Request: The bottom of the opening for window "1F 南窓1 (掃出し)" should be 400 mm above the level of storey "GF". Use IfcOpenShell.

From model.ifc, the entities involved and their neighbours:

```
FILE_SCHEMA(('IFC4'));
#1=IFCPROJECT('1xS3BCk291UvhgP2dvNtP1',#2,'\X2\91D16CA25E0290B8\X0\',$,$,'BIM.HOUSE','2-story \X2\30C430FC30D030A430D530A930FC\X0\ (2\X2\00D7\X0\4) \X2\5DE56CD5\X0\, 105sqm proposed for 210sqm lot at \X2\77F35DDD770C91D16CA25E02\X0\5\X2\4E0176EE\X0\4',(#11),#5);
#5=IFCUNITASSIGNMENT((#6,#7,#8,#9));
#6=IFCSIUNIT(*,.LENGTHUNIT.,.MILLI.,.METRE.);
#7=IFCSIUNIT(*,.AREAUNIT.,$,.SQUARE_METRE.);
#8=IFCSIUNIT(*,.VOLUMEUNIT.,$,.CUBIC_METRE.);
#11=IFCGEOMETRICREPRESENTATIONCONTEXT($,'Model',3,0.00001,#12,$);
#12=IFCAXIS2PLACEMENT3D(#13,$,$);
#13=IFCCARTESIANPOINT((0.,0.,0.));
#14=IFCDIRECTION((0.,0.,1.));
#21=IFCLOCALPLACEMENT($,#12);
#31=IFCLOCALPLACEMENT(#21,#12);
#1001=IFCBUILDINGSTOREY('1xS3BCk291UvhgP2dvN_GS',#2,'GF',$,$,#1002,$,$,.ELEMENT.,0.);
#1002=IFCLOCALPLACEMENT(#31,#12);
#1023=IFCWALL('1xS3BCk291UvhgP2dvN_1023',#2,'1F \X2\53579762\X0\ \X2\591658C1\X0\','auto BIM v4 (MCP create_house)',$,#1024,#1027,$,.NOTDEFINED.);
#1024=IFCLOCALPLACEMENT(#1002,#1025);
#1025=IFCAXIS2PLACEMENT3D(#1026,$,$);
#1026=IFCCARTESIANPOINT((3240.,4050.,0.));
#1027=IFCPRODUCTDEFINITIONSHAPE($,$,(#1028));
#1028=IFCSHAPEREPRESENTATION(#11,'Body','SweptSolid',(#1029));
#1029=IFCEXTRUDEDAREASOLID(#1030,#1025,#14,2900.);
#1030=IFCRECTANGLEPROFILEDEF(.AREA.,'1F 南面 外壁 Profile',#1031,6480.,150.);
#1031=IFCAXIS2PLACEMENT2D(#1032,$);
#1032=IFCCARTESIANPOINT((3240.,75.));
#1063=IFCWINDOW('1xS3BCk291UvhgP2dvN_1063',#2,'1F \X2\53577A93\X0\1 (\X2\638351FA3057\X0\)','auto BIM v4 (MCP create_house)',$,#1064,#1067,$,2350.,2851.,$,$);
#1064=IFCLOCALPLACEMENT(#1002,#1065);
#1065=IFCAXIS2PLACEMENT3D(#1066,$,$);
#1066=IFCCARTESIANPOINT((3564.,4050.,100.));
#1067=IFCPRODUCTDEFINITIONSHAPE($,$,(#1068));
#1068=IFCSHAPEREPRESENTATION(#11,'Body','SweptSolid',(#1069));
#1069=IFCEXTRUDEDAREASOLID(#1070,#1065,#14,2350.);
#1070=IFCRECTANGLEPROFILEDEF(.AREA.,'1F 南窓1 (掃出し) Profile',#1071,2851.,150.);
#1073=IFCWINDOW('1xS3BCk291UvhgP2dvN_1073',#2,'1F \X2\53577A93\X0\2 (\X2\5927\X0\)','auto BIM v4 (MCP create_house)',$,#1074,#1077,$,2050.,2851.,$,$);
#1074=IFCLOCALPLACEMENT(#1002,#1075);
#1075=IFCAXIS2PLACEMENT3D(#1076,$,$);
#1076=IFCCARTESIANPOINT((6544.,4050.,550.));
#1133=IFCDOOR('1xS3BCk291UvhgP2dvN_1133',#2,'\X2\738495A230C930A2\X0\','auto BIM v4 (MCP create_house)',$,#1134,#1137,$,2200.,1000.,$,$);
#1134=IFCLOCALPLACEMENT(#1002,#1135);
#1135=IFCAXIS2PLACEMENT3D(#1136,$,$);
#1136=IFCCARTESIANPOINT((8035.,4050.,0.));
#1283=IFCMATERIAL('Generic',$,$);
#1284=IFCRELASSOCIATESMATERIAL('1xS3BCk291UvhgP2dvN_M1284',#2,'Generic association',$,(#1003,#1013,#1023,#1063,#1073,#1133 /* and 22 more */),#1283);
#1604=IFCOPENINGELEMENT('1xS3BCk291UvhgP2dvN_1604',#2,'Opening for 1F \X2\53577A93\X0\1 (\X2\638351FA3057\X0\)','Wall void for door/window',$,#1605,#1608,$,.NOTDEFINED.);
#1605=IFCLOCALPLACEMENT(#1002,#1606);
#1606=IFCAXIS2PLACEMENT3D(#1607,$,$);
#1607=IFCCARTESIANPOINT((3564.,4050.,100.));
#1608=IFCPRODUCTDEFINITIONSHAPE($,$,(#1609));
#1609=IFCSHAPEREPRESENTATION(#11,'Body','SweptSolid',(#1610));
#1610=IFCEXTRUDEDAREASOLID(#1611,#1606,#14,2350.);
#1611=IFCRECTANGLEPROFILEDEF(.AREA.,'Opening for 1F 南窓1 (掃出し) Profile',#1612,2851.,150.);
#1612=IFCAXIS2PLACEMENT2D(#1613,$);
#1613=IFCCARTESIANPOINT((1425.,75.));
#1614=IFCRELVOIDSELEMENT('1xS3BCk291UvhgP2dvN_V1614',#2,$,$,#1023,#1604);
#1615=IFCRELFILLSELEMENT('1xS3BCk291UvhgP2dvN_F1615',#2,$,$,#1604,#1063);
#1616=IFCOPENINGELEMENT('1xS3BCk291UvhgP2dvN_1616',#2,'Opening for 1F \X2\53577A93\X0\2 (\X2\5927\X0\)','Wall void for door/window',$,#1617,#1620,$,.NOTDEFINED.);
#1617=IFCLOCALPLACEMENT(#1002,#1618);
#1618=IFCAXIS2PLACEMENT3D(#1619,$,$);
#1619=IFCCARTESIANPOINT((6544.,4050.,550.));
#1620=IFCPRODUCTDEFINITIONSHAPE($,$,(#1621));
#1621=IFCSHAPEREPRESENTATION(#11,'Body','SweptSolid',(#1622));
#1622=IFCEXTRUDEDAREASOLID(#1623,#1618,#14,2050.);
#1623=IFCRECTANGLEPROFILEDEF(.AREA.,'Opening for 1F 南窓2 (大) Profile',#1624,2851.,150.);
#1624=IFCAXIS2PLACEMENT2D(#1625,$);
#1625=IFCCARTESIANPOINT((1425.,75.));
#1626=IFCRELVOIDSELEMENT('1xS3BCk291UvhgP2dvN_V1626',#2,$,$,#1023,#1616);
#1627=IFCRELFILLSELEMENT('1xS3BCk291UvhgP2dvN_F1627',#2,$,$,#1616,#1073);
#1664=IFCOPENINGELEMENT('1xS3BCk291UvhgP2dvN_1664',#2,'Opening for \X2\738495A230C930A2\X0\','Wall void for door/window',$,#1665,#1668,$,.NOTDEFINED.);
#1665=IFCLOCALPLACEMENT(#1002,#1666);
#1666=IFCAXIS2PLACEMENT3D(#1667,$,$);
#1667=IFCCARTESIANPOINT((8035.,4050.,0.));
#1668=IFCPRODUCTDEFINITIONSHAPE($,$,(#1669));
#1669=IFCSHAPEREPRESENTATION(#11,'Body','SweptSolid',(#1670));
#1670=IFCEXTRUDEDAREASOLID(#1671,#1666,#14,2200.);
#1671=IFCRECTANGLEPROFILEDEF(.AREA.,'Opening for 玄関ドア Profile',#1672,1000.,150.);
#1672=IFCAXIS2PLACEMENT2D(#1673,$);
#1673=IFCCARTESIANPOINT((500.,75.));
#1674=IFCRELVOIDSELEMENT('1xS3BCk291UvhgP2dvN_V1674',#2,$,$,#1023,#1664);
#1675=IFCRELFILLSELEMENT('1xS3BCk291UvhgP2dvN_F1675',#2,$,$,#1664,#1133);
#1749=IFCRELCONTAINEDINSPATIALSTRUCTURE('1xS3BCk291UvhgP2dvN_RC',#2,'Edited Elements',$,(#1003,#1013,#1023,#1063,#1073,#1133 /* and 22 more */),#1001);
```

```python
import numpy as np
import ifcopenshell
import ifcopenshell.api.geometry
import ifcopenshell.geom
import ifcopenshell.util.element
import ifcopenshell.util.placement
import ifcopenshell.util.shape
import ifcopenshell.util.unit

model = ifcopenshell.open("model.ifc")
unit_scale = ifcopenshell.util.unit.calculate_unit_scale(model)

window = model.by_guid("1xS3BCk291UvhgP2dvN_1063")
opening = window.FillsVoids[0].RelatingOpeningElement
storey = ifcopenshell.util.element.get_container(window, ifc_class="IfcBuildingStorey")
level = ifcopenshell.util.placement.get_local_placement(storey.ObjectPlacement)[2, 3]

# The opening's origin need not be at the sill, so measure its lowest point.
shape = ifcopenshell.geom.create_shape(ifcopenshell.geom.settings(), opening)
bottom = ifcopenshell.util.shape.get_shape_bottom_elevation(shape, shape.geometry) / unit_scale
dz = level + 0.4 / unit_scale - bottom

shift = np.array([0.0, 0.0, dz])
# The window is not placed relative to its opening, so move both.
for product in (opening, window):
    matrix = ifcopenshell.util.placement.get_local_placement(product.ObjectPlacement)
    matrix[:3, 3] += shift
    ifcopenshell.api.geometry.edit_object_placement(model, product=product, matrix=matrix, is_si=False)

print(f"moved by {dz * unit_scale:+.3f} m")

model.write("model_edited.ifc")
```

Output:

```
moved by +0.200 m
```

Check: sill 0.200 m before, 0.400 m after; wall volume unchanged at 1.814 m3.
